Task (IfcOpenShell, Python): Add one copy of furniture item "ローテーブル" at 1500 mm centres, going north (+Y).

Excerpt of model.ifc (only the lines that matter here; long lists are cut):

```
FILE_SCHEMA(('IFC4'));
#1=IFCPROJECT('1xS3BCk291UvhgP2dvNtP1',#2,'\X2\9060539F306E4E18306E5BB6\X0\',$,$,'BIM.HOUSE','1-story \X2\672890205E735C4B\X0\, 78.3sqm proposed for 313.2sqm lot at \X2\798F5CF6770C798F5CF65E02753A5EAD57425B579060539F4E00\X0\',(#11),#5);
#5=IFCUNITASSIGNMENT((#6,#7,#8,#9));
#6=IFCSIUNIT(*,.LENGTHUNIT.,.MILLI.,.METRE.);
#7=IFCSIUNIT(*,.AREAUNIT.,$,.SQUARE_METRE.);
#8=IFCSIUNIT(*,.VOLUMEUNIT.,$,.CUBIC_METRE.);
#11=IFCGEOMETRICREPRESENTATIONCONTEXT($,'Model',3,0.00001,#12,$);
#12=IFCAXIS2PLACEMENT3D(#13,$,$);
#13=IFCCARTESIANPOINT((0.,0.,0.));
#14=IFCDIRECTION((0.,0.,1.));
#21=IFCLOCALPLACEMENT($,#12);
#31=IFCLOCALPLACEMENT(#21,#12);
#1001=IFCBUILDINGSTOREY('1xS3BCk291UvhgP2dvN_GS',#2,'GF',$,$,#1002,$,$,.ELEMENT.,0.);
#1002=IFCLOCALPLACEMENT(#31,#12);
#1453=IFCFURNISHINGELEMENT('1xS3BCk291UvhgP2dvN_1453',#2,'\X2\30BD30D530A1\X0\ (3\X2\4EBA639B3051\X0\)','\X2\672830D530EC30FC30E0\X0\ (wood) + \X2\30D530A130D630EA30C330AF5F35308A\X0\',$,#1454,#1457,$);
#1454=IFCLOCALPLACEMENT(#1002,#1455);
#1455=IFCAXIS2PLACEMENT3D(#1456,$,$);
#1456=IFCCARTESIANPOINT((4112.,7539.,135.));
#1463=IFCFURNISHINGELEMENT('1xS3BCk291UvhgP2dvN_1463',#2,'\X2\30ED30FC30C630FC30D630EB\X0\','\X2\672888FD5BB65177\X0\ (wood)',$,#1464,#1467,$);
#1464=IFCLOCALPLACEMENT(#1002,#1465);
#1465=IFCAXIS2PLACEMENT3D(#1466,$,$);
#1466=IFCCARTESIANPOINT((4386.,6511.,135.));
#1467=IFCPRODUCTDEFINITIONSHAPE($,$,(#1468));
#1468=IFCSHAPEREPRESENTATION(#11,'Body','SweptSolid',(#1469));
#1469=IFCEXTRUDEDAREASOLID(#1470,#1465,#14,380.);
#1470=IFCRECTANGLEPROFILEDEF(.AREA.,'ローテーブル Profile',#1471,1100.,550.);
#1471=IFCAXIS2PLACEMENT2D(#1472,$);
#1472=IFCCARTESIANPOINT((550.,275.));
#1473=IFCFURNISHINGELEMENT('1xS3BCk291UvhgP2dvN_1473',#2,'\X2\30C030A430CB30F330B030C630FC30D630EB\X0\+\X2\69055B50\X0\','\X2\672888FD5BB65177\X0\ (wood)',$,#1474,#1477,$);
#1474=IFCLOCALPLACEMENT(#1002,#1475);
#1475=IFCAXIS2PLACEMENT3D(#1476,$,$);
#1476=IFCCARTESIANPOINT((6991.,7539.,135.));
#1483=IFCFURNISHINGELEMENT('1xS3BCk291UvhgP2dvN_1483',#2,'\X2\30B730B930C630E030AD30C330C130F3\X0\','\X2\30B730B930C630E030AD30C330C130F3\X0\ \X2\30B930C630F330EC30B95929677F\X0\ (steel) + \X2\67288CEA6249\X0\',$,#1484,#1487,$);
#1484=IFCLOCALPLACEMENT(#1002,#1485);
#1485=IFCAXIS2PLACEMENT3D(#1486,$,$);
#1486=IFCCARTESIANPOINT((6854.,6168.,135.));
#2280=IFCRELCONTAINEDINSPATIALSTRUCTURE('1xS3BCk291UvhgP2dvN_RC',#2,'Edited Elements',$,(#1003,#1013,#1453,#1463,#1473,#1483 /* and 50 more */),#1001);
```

```python
import numpy as np
import ifcopenshell
import ifcopenshell.api.geometry
import ifcopenshell.api.root
import ifcopenshell.util.element
import ifcopenshell.util.placement
import ifcopenshell.util.unit

model = ifcopenshell.open("model.ifc")
unit_scale = ifcopenshell.util.unit.calculate_unit_scale(model)


def reuse_history(source, copy):
    """copy_class also copies each property set's owner history, people and application; keep the originals."""
    for rel in copy.IsDefinedBy:
        if rel.is_a("IfcRelDefinesByProperties") and (history := rel.RelatingPropertyDefinition.OwnerHistory):
            rel.RelatingPropertyDefinition.OwnerHistory = source.OwnerHistory
            ifcopenshell.util.element.remove_deep2(model, history)


source = model.by_guid("1xS3BCk291UvhgP2dvN_1463")
base = ifcopenshell.util.placement.get_local_placement(source.ObjectPlacement)
step = np.array([0.0, 1.0, 0.0]) * 1.5 / unit_scale

for i in range(1, 2):
    copy = ifcopenshell.api.root.copy_class(model, product=source)
    copy.Representation = ifcopenshell.util.element.copy_deep(
        model, source.Representation, exclude=["IfcGeometricRepresentationContext", "IfcRepresentationMap"]
    )
    reuse_history(source, copy)
    matrix = base.copy()
    matrix[:3, 3] += i * step
    print("added at", matrix[:3, 3].round(3) + 0.0)
    ifcopenshell.api.geometry.edit_object_placement(model, product=copy, matrix=matrix, is_si=False)

model.write("model_rev.ifc")
```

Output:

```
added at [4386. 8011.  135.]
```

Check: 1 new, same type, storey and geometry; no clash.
